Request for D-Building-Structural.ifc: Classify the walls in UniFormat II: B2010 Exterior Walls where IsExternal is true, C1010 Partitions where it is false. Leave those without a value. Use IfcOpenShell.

First a look at what the model holds.

```python
import ifcopenshell
import ifcopenshell.util.element

model = ifcopenshell.open("D-Building-Structural.ifc")
print(model.schema)
print("classifications:", [c.Name for c in model.by_type("IfcClassification")])
values = [ifcopenshell.util.element.get_pset(e, "Pset_WallCommon", "IsExternal") for e in model.by_type("IfcWall")]
for value in (True, False, None):
    print("IsExternal", value, values.count(value))
```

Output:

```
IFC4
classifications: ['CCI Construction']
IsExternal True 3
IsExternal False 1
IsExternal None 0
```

```python
import ifcopenshell
import ifcopenshell.api.classification
import ifcopenshell.util.element

model = ifcopenshell.open("D-Building-Structural.ifc")

system = ifcopenshell.api.classification.add_classification(model, classification="UniFormat II")

walls = model.by_type("IfcWall")
external = {e: ifcopenshell.util.element.get_pset(e, "Pset_WallCommon", "IsExternal") for e in walls}
for flag, code, name in ((True, "B2010", "Exterior Walls"), (False, "C1010", "Partitions")):
    products = [e for e in walls if external[e] is flag]
    ifcopenshell.api.classification.add_reference(
        model, products=products, classification=system, identification=code, name=name
    )
    print(code, len(products))

model.write("D-Building-Structural-out.ifc")
```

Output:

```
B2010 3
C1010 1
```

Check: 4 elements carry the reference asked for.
